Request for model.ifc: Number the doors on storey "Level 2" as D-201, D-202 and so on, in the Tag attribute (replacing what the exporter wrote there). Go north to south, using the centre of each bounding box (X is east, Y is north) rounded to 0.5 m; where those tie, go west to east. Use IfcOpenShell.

First a look at what the model holds.

```python
import ifcopenshell
import ifcopenshell.util.element
import ifcopenshell.util.placement

model = ifcopenshell.open("model.ifc")
print(model.schema)
storey = next(s for s in model.by_type("IfcBuildingStorey") if s.Name == "Level 2")
doors = [e for e in ifcopenshell.util.element.get_decomposition(storey) if e.is_a("IfcDoor")]
for e in sorted(doors, key=lambda e: e.id()):
    origin = ifcopenshell.util.placement.get_local_placement(e.ObjectPlacement)[:3, 3]
    print(e.id(), e.Tag, e.Name, origin.round(2) + 0.0, sep=" | ")
```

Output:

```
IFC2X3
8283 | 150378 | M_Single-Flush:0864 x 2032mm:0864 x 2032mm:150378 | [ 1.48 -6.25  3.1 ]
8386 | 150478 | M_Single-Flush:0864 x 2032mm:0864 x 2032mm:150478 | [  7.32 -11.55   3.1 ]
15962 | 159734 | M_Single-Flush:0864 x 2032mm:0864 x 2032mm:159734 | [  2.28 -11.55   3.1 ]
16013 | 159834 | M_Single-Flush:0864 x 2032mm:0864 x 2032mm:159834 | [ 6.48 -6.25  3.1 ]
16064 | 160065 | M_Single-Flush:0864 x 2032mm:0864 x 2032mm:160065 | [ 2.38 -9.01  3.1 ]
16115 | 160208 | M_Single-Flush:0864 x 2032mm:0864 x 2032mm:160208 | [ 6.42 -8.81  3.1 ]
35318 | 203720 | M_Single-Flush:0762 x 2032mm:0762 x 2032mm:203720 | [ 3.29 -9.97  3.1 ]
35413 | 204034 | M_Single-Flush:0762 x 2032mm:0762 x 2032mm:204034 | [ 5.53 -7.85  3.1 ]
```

```python
import ifcopenshell
import ifcopenshell.geom
import ifcopenshell.util.element
import ifcopenshell.util.shape

model = ifcopenshell.open("model.ifc")
settings = ifcopenshell.geom.settings()
settings.set("use-world-coords", True)


def centre(element):
    shape = ifcopenshell.geom.create_shape(settings, element)
    return ifcopenshell.util.shape.get_bbox_centroid(shape.geometry)


storey = next(s for s in model.by_type("IfcBuildingStorey") if s.Name == "Level 2")
doors = [e for e in ifcopenshell.util.element.get_decomposition(storey) if e.is_a("IfcDoor")]

# Insertion points can sit at a corner or the storey origin, so sort by the geometry (in metres).
centres = {e: centre(e) for e in doors}
doors.sort(key=lambda e: (-round(centres[e][1] / 0.5), centres[e][0]))

for i, e in enumerate(doors, start=1):
    number = f"D-2{i:02d}"
    e.Tag = number
    print(e.id(), number)

model.write("model-out.ifc")
```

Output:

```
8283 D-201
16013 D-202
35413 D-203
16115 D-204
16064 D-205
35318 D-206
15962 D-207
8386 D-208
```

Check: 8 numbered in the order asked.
